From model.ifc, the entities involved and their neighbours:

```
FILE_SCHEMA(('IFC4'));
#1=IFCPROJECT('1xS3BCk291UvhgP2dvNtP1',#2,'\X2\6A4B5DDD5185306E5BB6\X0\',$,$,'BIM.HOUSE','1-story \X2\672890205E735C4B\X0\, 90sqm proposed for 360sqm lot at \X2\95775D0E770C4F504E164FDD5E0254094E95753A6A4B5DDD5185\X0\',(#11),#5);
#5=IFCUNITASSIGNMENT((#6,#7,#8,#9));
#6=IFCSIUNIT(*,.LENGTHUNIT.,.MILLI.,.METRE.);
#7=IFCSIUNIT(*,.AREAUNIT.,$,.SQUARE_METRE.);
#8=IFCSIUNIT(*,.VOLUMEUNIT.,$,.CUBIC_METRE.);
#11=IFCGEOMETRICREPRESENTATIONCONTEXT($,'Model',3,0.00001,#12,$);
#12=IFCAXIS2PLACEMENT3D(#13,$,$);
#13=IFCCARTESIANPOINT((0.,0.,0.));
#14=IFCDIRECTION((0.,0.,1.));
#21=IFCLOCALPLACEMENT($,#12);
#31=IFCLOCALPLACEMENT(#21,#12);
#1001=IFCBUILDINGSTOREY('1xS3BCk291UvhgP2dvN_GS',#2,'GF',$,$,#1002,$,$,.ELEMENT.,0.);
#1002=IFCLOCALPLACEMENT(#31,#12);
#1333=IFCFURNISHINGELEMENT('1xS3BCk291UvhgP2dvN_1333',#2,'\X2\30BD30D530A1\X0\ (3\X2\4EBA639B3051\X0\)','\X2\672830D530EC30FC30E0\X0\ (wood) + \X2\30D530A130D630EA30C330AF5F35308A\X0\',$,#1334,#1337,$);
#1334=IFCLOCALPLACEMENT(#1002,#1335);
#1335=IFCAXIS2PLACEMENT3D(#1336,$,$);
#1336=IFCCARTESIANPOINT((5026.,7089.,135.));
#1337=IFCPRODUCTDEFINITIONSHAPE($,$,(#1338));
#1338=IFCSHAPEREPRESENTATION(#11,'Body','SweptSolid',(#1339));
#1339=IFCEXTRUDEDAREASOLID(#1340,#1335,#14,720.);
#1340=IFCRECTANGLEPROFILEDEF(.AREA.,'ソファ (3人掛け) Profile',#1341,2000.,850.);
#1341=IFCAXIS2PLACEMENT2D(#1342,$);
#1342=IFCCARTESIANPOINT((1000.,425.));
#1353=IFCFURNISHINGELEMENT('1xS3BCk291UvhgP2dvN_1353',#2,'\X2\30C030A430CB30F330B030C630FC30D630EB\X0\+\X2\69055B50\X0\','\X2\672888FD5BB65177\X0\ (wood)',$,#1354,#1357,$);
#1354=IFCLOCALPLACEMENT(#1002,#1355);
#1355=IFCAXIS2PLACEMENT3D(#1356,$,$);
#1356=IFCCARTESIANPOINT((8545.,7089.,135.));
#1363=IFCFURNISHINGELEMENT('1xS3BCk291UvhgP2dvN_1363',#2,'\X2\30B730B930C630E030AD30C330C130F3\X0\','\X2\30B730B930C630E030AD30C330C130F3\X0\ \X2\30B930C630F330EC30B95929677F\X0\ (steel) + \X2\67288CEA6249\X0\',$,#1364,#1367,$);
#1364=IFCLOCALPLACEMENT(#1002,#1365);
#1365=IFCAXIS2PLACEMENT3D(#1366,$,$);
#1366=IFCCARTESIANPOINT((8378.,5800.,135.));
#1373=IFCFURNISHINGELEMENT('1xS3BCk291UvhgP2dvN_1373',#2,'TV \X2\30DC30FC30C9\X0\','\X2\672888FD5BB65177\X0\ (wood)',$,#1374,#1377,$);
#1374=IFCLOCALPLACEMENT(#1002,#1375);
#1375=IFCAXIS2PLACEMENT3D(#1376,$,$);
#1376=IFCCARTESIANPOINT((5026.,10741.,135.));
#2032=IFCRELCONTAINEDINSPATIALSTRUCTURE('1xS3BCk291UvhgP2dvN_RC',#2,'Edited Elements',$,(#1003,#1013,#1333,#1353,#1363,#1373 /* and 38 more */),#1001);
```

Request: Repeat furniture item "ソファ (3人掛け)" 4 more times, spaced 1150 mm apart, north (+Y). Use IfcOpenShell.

```python
import numpy as np
import ifcopenshell
import ifcopenshell.api.geometry
import ifcopenshell.api.root
import ifcopenshell.util.element
import ifcopenshell.util.placement

model = ifcopenshell.open("model.ifc")


def reuse_history(source, copy):
    """copy_class also copies each property set's owner history, people and application; keep the originals."""
    for rel in copy.IsDefinedBy:
        if rel.is_a("IfcRelDefinesByProperties") and (history := rel.RelatingPropertyDefinition.OwnerHistory):
            rel.RelatingPropertyDefinition.OwnerHistory = source.OwnerHistory
            ifcopenshell.util.element.remove_deep2(model, history)


source = model.by_guid("1xS3BCk291UvhgP2dvN_1333")
base = ifcopenshell.util.placement.get_local_placement(source.ObjectPlacement)
step = np.array([0.0, 1.0, 0.0]) * 1150.0

for i in range(1, 5):
    copy = ifcopenshell.api.root.copy_class(model, product=source)
    copy.Representation = ifcopenshell.util.element.copy_deep(
        model, source.Representation, exclude=["IfcGeometricRepresentationContext", "IfcRepresentationMap"]
    )
    reuse_history(source, copy)
    matrix = base.copy()
    matrix[:3, 3] += i * step
    print("added at", matrix[:3, 3].round(3) + 0.0)
    ifcopenshell.api.geometry.edit_object_placement(model, product=copy, matrix=matrix, is_si=False)

model.write("model_v2.ifc")
```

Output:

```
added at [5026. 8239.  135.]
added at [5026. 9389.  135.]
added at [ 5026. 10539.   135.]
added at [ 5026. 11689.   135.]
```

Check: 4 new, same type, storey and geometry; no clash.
